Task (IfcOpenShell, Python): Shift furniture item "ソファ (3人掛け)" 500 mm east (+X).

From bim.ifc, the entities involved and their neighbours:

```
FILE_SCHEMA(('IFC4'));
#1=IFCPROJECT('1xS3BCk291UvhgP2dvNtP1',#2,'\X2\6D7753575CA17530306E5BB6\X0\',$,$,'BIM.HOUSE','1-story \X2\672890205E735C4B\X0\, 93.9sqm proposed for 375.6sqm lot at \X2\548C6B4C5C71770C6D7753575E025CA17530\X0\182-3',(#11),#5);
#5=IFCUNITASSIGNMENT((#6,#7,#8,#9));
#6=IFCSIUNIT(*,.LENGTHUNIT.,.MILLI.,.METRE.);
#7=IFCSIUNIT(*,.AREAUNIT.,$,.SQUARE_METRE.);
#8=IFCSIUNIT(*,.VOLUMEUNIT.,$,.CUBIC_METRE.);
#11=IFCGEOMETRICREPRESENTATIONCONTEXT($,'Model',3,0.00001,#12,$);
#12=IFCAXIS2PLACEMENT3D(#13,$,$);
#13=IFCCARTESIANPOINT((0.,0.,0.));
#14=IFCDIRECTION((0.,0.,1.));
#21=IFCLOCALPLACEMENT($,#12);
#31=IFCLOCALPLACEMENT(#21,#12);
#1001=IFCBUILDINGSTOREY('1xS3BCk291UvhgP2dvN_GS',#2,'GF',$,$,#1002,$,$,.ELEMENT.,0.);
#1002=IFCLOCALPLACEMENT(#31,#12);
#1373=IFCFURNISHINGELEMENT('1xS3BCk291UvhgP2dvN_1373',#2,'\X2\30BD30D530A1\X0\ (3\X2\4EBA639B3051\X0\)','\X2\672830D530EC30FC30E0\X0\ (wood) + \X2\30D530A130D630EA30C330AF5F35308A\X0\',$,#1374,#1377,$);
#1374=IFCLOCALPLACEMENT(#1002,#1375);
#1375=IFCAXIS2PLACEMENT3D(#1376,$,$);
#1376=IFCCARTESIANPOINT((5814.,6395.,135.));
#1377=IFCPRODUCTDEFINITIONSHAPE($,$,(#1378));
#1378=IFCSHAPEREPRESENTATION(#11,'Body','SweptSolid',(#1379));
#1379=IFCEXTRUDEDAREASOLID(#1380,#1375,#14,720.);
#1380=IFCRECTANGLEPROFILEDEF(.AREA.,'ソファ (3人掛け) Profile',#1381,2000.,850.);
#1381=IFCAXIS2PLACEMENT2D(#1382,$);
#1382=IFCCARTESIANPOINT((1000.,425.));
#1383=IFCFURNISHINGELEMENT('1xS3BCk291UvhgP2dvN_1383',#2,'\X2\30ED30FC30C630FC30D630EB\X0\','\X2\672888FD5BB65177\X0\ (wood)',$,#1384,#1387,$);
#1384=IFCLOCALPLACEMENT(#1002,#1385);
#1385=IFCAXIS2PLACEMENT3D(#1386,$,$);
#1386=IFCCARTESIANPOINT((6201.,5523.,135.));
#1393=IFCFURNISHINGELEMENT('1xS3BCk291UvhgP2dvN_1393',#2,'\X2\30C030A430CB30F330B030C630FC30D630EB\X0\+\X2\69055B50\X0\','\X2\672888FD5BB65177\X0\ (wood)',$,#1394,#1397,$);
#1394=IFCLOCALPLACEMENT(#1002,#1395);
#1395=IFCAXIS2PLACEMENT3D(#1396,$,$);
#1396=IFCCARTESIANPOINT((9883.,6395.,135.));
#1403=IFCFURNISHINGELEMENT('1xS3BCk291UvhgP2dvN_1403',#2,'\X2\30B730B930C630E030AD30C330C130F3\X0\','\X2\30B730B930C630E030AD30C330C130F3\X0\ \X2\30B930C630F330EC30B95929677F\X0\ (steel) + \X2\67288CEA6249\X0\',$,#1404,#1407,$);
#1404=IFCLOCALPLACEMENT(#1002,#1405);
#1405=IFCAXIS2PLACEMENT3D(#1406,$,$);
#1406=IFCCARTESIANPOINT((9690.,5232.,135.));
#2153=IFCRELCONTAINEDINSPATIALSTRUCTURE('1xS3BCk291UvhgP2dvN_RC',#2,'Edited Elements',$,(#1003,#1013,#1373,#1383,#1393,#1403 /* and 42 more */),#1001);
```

```python
import ifcopenshell
import ifcopenshell.api.geometry
import ifcopenshell.util.placement
import ifcopenshell.util.unit

model = ifcopenshell.open("bim.ifc")
unit_scale = ifcopenshell.util.unit.calculate_unit_scale(model)

item = model.by_id(1373)
matrix = ifcopenshell.util.placement.get_local_placement(item.ObjectPlacement)
matrix[0, 3] += 0.5 / unit_scale
ifcopenshell.api.geometry.edit_object_placement(model, product=item, matrix=matrix, is_si=False)

print(ifcopenshell.util.placement.get_local_placement(item.ObjectPlacement).round(3) + 0.0)

model.write("bim_edited.ifc")
```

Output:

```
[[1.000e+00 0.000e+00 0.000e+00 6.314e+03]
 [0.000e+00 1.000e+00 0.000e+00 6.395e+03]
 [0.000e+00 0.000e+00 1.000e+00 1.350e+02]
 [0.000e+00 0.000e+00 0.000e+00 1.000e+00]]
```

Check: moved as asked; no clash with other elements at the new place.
